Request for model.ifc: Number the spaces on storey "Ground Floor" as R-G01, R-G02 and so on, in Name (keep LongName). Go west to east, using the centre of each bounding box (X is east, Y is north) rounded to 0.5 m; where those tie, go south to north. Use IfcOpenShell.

First a look at what the model holds.

```python
import ifcopenshell
import ifcopenshell.util.element
import ifcopenshell.util.placement

model = ifcopenshell.open("model.ifc")
print(model.schema)
storey = next(s for s in model.by_type("IfcBuildingStorey") if s.Name == "Ground Floor")
spaces = [e for e in ifcopenshell.util.element.get_decomposition(storey) if e.is_a("IfcSpace")]
for e in sorted(spaces, key=lambda e: e.id()):
    origin = ifcopenshell.util.placement.get_local_placement(e.ObjectPlacement)[:3, 3]
    print(e.id(), e.Name, e.LongName, origin.round(2) + 0.0, sep=" | ")
```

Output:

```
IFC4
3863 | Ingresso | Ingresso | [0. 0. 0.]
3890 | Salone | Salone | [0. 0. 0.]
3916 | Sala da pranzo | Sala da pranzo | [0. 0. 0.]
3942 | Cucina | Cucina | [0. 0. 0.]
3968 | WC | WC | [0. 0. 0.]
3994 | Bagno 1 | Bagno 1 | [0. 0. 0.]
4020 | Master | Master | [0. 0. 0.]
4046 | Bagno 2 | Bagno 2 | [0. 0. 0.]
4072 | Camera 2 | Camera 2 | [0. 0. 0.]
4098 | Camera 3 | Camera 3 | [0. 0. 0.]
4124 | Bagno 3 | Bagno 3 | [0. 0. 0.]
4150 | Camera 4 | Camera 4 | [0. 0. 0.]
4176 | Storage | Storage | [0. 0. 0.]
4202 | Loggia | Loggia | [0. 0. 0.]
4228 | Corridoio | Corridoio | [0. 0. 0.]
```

```python
import ifcopenshell
import ifcopenshell.geom
import ifcopenshell.util.element
import ifcopenshell.util.shape

model = ifcopenshell.open("model.ifc")
settings = ifcopenshell.geom.settings()
settings.set("use-world-coords", True)


def centre(element):
    shape = ifcopenshell.geom.create_shape(settings, element)
    return ifcopenshell.util.shape.get_bbox_centroid(shape.geometry)


storey = next(s for s in model.by_type("IfcBuildingStorey") if s.Name == "Ground Floor")
spaces = [e for e in ifcopenshell.util.element.get_decomposition(storey) if e.is_a("IfcSpace")]

# Insertion points can sit at a corner or the storey origin, so sort by the geometry (in metres).
centres = {e: centre(e) for e in spaces}
spaces.sort(key=lambda e: (round(centres[e][0] / 0.5), centres[e][1]))

for i, e in enumerate(spaces, start=1):
    number = f"R-G{i:02d}"
    e.Name = number
    print(e.id(), number)

model.write("model_v2.ifc")
```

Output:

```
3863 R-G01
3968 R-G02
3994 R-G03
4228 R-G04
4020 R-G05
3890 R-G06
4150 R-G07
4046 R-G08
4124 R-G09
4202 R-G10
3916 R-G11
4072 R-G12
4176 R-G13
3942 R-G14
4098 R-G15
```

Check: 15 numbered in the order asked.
